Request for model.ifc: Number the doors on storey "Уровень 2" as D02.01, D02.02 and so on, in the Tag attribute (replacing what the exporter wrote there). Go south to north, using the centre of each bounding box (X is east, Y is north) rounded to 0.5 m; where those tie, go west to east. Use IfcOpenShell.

First a look at what the model holds.

```python
import ifcopenshell
import ifcopenshell.util.element
import ifcopenshell.util.placement

model = ifcopenshell.open("model.ifc")
print(model.schema)
storey = next(s for s in model.by_type("IfcBuildingStorey") if s.Name == "Уровень 2")
doors = [e for e in ifcopenshell.util.element.get_decomposition(storey) if e.is_a("IfcDoor")]
for e in sorted(doors, key=lambda e: e.id()):
    origin = ifcopenshell.util.placement.get_local_placement(e.ObjectPlacement)[:3, 3]
    print(e.id(), e.Tag, e.Name, origin.round(2) + 0.0, sep=" | ")
```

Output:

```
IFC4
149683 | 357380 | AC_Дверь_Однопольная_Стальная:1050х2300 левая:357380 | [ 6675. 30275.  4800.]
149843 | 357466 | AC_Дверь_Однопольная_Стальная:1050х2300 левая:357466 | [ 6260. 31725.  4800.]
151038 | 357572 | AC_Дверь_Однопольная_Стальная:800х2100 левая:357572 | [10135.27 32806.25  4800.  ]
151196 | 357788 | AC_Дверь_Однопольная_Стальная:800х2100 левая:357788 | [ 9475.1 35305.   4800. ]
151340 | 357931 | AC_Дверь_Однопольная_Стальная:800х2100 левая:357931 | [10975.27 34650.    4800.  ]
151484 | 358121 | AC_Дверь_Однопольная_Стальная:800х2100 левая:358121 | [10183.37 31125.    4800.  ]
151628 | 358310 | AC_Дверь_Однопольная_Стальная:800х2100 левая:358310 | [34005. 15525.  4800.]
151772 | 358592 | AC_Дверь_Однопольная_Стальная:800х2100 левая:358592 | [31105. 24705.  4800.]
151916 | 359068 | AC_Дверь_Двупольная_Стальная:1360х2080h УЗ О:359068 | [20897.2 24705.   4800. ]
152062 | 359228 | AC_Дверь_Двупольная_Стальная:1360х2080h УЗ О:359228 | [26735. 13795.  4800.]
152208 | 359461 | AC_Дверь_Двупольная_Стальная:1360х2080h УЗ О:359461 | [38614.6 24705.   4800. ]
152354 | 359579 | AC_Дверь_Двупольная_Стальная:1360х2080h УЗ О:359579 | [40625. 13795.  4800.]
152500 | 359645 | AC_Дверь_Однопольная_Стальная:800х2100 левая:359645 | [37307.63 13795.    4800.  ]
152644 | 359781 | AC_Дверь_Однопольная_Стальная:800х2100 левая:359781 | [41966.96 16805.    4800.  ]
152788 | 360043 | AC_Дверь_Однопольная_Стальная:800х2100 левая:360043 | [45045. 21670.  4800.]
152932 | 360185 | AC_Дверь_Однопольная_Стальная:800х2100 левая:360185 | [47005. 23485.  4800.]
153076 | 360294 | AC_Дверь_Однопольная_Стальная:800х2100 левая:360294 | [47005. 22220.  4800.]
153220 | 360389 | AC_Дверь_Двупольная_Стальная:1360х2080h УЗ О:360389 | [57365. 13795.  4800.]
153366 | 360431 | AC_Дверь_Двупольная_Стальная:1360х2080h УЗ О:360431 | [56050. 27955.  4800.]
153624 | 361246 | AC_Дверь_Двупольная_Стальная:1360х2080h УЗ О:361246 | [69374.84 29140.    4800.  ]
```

```python
import ifcopenshell
import ifcopenshell.geom
import ifcopenshell.util.element
import ifcopenshell.util.shape

model = ifcopenshell.open("model.ifc")
settings = ifcopenshell.geom.settings()
settings.set("use-world-coords", True)


def centre(element):
    shape = ifcopenshell.geom.create_shape(settings, element)
    return ifcopenshell.util.shape.get_bbox_centroid(shape.geometry)


storey = next(s for s in model.by_type("IfcBuildingStorey") if s.Name == "Уровень 2")
doors = [e for e in ifcopenshell.util.element.get_decomposition(storey) if e.is_a("IfcDoor")]

# Insertion points can sit at a corner or the storey origin, so sort by the geometry (in metres).
centres = {e: centre(e) for e in doors}
doors.sort(key=lambda e: (round(centres[e][1] / 0.5), centres[e][0]))

for i, e in enumerate(doors, start=1):
    number = f"D02.{i:02d}"
    e.Tag = number
    print(e.id(), number)

model.write("model_updated.ifc")
```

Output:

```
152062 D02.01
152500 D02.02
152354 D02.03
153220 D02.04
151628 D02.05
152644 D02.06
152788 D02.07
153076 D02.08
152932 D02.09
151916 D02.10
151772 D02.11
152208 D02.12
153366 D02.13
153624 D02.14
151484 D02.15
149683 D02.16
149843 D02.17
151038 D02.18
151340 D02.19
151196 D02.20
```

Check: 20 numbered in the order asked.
